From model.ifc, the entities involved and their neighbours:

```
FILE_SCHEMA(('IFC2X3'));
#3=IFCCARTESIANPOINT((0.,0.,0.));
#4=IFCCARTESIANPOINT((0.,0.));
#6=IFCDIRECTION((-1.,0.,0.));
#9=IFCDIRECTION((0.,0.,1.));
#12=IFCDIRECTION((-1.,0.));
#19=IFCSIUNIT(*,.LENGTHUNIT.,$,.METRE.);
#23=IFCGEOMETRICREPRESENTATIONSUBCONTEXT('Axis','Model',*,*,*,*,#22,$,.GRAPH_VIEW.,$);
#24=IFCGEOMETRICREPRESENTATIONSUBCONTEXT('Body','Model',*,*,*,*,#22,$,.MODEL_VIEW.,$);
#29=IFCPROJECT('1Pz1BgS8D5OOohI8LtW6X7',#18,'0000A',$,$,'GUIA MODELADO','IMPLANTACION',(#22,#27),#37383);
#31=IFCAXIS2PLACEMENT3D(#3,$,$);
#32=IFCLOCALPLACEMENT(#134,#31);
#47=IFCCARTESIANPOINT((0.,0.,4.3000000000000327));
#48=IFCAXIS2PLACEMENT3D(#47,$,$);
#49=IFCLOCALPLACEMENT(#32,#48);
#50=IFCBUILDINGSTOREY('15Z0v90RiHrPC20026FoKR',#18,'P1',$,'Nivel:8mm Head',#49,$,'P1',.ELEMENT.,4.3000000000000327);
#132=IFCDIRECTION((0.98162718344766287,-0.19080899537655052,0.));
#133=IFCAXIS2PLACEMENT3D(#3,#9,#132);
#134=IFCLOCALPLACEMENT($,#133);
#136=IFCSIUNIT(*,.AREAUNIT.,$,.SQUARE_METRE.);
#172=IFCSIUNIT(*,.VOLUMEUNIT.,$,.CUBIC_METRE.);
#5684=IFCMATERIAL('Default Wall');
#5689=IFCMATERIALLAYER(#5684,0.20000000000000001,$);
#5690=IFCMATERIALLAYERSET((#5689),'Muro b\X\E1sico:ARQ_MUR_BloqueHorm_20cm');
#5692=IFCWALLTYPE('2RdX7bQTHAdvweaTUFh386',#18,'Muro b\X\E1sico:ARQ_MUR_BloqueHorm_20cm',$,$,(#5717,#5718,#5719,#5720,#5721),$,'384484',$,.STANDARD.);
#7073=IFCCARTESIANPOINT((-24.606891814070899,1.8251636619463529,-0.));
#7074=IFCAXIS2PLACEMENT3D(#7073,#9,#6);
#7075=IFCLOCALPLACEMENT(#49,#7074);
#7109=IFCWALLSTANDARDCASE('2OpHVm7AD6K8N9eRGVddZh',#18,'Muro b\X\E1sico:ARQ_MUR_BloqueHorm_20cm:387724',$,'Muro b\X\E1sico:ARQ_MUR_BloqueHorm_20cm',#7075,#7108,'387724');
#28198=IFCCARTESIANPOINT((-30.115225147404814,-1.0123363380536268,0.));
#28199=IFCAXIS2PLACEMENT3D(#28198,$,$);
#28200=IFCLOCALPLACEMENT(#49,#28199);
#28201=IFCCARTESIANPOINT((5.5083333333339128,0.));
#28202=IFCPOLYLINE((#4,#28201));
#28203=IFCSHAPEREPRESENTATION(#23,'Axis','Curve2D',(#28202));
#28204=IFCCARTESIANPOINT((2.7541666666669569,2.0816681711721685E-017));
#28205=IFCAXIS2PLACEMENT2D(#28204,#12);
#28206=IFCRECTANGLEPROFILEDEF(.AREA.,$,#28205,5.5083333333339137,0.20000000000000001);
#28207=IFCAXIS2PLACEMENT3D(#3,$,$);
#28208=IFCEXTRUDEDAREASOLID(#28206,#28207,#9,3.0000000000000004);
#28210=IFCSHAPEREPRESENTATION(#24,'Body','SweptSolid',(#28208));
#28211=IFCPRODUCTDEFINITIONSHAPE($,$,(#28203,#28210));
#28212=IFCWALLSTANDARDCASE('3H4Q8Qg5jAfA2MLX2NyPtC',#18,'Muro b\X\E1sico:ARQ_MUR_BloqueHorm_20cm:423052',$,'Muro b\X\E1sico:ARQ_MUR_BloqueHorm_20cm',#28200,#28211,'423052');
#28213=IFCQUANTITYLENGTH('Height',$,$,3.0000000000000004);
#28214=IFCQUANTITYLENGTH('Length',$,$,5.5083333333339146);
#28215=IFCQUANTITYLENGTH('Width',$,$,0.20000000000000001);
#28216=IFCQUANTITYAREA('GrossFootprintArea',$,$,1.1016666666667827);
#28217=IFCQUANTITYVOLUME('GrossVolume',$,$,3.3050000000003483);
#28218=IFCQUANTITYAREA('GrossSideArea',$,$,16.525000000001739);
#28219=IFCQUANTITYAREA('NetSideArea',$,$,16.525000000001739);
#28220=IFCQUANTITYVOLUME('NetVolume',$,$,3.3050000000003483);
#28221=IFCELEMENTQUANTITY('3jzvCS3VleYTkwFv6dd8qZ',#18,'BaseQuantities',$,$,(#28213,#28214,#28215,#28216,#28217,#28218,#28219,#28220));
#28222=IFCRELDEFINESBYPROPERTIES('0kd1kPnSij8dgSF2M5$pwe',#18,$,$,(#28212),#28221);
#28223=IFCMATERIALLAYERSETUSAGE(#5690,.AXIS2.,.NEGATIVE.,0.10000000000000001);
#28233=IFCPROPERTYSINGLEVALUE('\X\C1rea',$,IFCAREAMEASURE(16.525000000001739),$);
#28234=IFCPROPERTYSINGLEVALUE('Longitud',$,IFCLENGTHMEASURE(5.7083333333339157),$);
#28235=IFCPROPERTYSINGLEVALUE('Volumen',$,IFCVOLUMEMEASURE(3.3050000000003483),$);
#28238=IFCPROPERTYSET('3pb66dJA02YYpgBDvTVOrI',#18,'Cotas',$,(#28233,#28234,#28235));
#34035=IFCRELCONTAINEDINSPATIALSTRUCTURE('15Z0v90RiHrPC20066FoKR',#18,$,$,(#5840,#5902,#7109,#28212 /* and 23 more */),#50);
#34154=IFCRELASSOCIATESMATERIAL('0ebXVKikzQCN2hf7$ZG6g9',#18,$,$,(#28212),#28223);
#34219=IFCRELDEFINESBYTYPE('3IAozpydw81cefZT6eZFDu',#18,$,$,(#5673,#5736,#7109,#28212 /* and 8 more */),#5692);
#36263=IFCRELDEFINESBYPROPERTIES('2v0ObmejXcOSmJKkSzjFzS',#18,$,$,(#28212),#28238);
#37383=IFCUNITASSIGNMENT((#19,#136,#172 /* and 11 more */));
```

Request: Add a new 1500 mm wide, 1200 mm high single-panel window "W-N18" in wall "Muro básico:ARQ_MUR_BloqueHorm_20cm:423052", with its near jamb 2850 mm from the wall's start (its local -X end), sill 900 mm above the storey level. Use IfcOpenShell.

```python
import numpy as np
import ifcopenshell
import ifcopenshell.api.feature
import ifcopenshell.api.geometry
import ifcopenshell.api.pset
import ifcopenshell.api.root
import ifcopenshell.api.spatial
import ifcopenshell.api.type
import ifcopenshell.geom
import ifcopenshell.util.element
import ifcopenshell.util.placement
import ifcopenshell.util.representation
import ifcopenshell.util.shape
import ifcopenshell.util.unit

model = ifcopenshell.open("model.ifc")
unit_scale = ifcopenshell.util.unit.calculate_unit_scale(model)
area_scale = ifcopenshell.util.unit.calculate_unit_scale(model, "AREAUNIT")
volume_scale = ifcopenshell.util.unit.calculate_unit_scale(model, "VOLUMEUNIT")
settings = ifcopenshell.geom.settings()


def volume(element):
    """Net volume in cubic metres, openings subtracted."""
    shape = ifcopenshell.geom.create_shape(settings, element)
    return ifcopenshell.util.shape.get_volume(shape.geometry)


wall = model.by_id(28212)
storey = ifcopenshell.util.element.get_container(wall, ifc_class="IfcBuildingStorey")
context = ifcopenshell.util.representation.get_context(model, "Model", "Body", "MODEL_VIEW")
before = volume(wall)

width, height, from_end, sill = 1.5, 1.2, 2.85, 0.9  # metres

# The wall runs along its own X axis, and the end named is its -X end.
wall_shape = ifcopenshell.geom.create_shape(settings, wall)
x, y, z = ifcopenshell.util.shape.get_vertices(wall_shape.geometry).T
start = x.min() + from_end
face, thickness = float(y.min()), float(y.max() - y.min())
wall_matrix = ifcopenshell.util.placement.get_local_placement(wall.ObjectPlacement)
level = ifcopenshell.util.placement.get_local_placement(storey.ObjectPlacement)[2, 3]


def in_wall(x, y):
    """Placement at x, y metres in the wall's axes, at sill height."""
    matrix = wall_matrix.copy()
    matrix[:, 3] = wall_matrix @ np.array([x / unit_scale, y / unit_scale, 0.0, 1.0])
    matrix[2, 3] = level + sill / unit_scale
    return matrix


# Opening: a box that overshoots both wall faces by 50 mm.
opening = ifcopenshell.api.root.create_entity(model, ifc_class="IfcOpeningElement")
box = ifcopenshell.api.geometry.add_wall_representation(
    model, context=context, length=width, height=height, thickness=thickness + 0.1
)
ifcopenshell.api.geometry.assign_representation(model, product=opening, representation=box)
ifcopenshell.api.geometry.edit_object_placement(model, product=opening, matrix=in_wall(start, face - 0.05), is_si=False)
ifcopenshell.api.feature.add_feature(model, feature=opening, element=wall)

window = ifcopenshell.api.root.create_entity(model, ifc_class="IfcWindow", name="W-N18")
window.OverallWidth, window.OverallHeight = width / unit_scale, height / unit_scale
body = ifcopenshell.api.geometry.add_window_representation(
    model,
    context=context,
    overall_width=window.OverallWidth,
    overall_height=window.OverallHeight,
    partition_type="SINGLE_PANEL",
)
ifcopenshell.api.geometry.assign_representation(model, product=window, representation=body)
ifcopenshell.api.spatial.assign_container(model, products=[window], relating_structure=storey)
fills = ifcopenshell.api.feature.add_filling(model, opening=opening, element=window)
fills.OwnerHistory = window.OwnerHistory  # required in IFC2X3

# IFC2X3 keeps the operation on the window style.
style = ifcopenshell.api.root.create_entity(model, ifc_class="IfcWindowStyle", name="W-N18")
style.OperationType, style.ConstructionType = "SINGLE_PANEL", "NOTDEFINED"
style.ParameterTakesPrecedence = style.Sizeable = False
ifcopenshell.api.type.assign_type(model, related_objects=[window], relating_type=style)

# Centre the window in the wall's thickness.
ifcopenshell.api.geometry.edit_object_placement(model, product=window, matrix=in_wall(start, face), is_si=False)
window_shape = ifcopenshell.geom.create_shape(settings, window)
depth = ifcopenshell.util.shape.get_vertices(window_shape.geometry)[:, 1]
offset = face + thickness / 2 - (depth.min() + depth.max()) / 2
ifcopenshell.api.geometry.edit_object_placement(model, product=window, matrix=in_wall(start, offset), is_si=False)

after = volume(wall)

# Update the wall's stored quantities.
qto = model.by_id(ifcopenshell.util.element.get_pset(wall, "BaseQuantities", should_inherit=False)["id"])
ifcopenshell.api.pset.edit_qto(model, qto=qto, properties={
    "NetSideArea": after / thickness / area_scale,
    "NetVolume": after / volume_scale,
})
pset = model.by_id(ifcopenshell.util.element.get_pset(wall, "Cotas", should_inherit=False)["id"])
ifcopenshell.api.pset.edit_pset(model, pset=pset, properties={
    "Área": model.create_entity("IfcAreaMeasure", after / thickness / area_scale),
    "Volumen": model.create_entity("IfcVolumeMeasure", after / volume_scale),
})

print(f"wall volume {before:.3f} -> {after:.3f} m3")

model.write("model_edited.ifc")
```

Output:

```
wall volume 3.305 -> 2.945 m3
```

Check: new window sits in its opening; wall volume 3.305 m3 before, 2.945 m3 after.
